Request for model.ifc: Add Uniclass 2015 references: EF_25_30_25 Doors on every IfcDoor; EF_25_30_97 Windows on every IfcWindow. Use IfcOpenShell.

First a look at what the model holds.

```python
import ifcopenshell

model = ifcopenshell.open("model.ifc")
print(model.schema)
print("classifications:", [c.Name for c in model.by_type("IfcClassification")])
for ifc_class in ("IfcDoor", "IfcRoof", "IfcStair", "IfcWall", "IfcWindow"):
    print(ifc_class, len(model.by_type(ifc_class)))
```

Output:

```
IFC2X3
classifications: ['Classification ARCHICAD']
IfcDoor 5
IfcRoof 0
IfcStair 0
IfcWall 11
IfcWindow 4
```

```python
import ifcopenshell
import ifcopenshell.api.classification

model = ifcopenshell.open("model.ifc")

# IFC2X3 requires Source and Edition and has no link from the project to the system.
system = model.create_entity("IfcClassification", Source="NBS", Edition="2015", Name="Uniclass 2015")

codes = {
    "IfcDoor": ("EF_25_30_25", "Doors"),
    "IfcWindow": ("EF_25_30_97", "Windows"),
}
for ifc_class, (code, name) in codes.items():
    products = model.by_type(ifc_class)
    ifcopenshell.api.classification.add_reference(
        model, products=products, classification=system, identification=code, name=name
    )
    print(code, len(products))

model.write("model-out.ifc")
```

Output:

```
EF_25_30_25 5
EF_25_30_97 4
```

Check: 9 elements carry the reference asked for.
